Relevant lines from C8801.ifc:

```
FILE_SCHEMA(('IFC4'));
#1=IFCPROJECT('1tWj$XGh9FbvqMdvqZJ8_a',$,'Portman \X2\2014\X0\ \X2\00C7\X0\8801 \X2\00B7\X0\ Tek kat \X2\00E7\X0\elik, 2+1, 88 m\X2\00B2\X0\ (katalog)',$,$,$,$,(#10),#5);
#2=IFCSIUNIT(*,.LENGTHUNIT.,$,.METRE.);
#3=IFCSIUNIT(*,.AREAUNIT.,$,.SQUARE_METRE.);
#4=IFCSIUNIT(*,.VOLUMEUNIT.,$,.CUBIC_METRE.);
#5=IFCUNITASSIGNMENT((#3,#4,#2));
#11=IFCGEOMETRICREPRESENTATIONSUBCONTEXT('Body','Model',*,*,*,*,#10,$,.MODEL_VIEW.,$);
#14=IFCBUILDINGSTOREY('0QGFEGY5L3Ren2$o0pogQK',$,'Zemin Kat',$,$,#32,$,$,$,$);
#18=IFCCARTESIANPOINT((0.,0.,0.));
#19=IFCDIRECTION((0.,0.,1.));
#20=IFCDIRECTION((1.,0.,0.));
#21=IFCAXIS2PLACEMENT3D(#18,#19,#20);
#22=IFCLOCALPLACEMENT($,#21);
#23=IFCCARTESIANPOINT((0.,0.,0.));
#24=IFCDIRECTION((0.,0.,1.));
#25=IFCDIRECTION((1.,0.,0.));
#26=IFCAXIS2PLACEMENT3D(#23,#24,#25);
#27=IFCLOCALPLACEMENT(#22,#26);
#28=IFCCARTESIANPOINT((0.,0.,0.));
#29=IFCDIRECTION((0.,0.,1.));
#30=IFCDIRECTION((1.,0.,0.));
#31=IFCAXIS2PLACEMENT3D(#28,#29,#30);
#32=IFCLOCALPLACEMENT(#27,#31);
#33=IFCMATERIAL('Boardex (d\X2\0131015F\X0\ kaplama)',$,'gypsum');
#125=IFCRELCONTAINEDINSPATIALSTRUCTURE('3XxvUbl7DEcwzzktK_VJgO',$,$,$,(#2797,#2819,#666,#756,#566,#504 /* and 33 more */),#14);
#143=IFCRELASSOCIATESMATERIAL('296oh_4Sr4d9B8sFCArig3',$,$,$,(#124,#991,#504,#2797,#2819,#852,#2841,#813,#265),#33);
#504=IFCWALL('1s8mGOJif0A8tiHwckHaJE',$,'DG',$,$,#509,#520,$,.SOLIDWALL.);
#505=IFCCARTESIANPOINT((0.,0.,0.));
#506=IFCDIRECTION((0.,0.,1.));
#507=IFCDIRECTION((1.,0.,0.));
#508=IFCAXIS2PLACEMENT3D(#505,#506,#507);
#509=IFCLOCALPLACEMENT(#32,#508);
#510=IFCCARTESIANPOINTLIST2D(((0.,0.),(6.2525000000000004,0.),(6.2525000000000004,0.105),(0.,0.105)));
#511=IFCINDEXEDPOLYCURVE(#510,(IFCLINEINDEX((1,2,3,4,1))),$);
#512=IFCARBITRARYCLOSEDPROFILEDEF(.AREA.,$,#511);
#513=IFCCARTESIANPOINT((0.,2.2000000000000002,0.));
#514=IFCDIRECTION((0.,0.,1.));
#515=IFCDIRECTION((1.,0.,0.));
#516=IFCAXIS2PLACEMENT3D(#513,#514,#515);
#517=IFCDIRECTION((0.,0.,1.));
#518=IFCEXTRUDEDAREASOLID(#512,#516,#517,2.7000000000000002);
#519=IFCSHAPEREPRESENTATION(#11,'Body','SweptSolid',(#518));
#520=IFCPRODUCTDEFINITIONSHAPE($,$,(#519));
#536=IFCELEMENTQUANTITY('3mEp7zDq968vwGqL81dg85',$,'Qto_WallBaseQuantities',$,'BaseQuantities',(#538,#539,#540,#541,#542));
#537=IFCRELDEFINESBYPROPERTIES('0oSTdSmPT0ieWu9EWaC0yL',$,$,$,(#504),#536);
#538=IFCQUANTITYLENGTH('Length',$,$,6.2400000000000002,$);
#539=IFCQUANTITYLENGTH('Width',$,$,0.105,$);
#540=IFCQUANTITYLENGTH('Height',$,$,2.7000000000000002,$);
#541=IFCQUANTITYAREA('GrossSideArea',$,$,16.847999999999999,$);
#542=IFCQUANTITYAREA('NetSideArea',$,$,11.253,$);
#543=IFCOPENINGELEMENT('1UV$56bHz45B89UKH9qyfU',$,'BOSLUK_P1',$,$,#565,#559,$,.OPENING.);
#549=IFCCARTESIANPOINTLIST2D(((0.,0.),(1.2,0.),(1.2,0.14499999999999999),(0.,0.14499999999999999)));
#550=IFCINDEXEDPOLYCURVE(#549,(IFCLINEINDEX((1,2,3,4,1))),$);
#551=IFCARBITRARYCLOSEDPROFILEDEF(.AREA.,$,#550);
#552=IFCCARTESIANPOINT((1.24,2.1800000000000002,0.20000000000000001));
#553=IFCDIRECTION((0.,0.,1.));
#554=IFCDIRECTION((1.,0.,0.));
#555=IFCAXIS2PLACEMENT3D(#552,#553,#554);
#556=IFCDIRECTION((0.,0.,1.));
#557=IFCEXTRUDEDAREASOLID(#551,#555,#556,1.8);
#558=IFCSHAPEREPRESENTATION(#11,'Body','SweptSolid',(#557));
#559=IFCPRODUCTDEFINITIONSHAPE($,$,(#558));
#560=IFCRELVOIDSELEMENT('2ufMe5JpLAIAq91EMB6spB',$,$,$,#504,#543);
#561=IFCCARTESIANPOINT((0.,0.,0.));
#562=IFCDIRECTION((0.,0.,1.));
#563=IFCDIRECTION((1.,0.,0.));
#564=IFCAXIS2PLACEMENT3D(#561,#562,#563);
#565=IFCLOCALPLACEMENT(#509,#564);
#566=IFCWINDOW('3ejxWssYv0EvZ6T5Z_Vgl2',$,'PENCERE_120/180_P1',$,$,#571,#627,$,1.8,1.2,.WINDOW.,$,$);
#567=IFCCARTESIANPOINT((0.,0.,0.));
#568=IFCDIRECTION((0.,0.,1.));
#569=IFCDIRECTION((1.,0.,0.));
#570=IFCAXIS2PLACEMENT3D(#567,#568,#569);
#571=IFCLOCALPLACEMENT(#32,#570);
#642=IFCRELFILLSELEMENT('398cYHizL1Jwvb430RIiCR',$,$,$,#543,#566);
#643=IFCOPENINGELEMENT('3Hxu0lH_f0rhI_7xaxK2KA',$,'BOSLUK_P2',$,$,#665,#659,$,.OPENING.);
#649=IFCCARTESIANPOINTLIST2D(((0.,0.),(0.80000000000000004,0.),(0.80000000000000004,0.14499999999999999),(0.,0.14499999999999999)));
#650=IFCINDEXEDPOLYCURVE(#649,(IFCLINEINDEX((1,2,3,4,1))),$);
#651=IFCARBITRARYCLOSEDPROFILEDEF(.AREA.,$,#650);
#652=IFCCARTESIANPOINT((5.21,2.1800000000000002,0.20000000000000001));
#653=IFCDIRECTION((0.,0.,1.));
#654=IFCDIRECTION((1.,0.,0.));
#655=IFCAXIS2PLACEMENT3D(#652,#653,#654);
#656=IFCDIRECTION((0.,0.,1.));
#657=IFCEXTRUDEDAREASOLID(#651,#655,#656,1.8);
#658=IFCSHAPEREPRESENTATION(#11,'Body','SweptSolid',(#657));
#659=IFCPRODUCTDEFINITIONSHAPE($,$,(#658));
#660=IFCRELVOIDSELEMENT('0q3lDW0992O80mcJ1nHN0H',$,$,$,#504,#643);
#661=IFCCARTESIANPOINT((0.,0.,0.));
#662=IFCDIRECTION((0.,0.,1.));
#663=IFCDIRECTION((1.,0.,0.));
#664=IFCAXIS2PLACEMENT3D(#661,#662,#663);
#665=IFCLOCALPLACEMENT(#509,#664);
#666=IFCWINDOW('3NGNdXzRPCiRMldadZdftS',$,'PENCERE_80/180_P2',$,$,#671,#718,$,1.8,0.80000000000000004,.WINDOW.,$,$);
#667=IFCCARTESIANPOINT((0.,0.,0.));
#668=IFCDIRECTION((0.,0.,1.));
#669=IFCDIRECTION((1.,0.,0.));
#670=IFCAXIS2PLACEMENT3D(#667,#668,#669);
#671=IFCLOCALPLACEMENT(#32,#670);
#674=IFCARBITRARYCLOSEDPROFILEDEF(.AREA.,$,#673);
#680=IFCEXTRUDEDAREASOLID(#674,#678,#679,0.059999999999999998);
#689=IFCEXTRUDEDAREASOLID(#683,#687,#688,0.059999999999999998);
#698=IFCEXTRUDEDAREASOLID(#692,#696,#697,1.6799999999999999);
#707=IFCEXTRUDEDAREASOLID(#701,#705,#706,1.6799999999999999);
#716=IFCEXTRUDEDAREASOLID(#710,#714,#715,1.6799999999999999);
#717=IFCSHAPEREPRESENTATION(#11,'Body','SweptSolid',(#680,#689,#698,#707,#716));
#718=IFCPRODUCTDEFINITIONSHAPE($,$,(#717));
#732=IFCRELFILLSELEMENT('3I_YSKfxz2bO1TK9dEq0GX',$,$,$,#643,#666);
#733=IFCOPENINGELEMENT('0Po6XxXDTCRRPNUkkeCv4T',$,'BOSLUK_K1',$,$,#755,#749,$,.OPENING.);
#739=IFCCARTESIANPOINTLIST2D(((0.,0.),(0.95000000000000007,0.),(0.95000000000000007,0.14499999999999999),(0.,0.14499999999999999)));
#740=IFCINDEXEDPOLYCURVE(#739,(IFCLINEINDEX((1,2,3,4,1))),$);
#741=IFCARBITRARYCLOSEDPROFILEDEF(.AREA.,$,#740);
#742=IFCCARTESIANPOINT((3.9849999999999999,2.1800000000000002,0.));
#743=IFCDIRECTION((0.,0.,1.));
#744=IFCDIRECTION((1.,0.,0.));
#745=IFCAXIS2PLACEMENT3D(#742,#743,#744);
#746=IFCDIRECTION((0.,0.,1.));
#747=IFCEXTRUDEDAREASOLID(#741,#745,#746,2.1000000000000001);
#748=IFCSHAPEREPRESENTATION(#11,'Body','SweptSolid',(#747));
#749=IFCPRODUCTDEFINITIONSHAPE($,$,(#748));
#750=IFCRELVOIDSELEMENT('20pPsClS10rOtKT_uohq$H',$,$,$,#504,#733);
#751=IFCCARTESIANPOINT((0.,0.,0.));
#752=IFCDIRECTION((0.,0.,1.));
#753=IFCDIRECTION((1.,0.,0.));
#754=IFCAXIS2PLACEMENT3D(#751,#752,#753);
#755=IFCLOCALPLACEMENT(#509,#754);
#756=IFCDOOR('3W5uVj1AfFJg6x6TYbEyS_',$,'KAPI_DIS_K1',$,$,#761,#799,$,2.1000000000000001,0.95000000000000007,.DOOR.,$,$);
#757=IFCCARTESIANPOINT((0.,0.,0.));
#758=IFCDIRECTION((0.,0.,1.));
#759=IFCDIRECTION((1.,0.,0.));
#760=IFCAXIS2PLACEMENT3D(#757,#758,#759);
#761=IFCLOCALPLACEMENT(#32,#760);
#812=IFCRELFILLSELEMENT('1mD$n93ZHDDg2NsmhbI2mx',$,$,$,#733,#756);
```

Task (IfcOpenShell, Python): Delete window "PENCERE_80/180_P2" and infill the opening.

```python
import ifcopenshell
import ifcopenshell.api.feature
import ifcopenshell.api.pset
import ifcopenshell.api.root
import ifcopenshell.geom
import ifcopenshell.util.element
import ifcopenshell.util.shape
import ifcopenshell.util.unit

model = ifcopenshell.open("C8801.ifc")
area_scale = ifcopenshell.util.unit.calculate_unit_scale(model, "AREAUNIT")
settings = ifcopenshell.geom.settings()


def volume(element):
    """Net volume in cubic metres, openings subtracted."""
    shape = ifcopenshell.geom.create_shape(settings, element)
    return ifcopenshell.util.shape.get_volume(shape.geometry)


window = model.by_id(666)
opening = window.FillsVoids[0].RelatingOpeningElement
wall = opening.VoidsElements[0].RelatingBuildingElement
before = volume(wall)

ifcopenshell.api.root.remove_product(model, product=window)
ifcopenshell.api.feature.remove_feature(model, feature=opening)

after = volume(wall)
thickness = 0.105  # wall thickness in metres

# Update the wall's stored quantities.
qto = model.by_id(ifcopenshell.util.element.get_pset(wall, "Qto_WallBaseQuantities", should_inherit=False)["id"])
ifcopenshell.api.pset.edit_qto(model, qto=qto, properties={"NetSideArea": after / thickness / area_scale})

print(f"wall volume {before:.3f} -> {after:.3f} m3")

model.write("C8801_v2.ifc")
```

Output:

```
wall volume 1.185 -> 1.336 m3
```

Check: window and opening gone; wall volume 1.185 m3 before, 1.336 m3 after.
